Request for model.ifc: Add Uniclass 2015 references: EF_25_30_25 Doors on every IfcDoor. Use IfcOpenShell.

First a look at what the model holds.

```python
import ifcopenshell

model = ifcopenshell.open("model.ifc")
print(model.schema)
print("classifications:", [c.Name for c in model.by_type("IfcClassification")])
for ifc_class in ("IfcDoor", "IfcRoof", "IfcStair", "IfcWall", "IfcWindow"):
    print(ifc_class, len(model.by_type(ifc_class)))
```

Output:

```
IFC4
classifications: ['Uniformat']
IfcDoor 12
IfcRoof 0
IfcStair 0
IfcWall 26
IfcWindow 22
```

```python
import ifcopenshell
import ifcopenshell.api.classification

model = ifcopenshell.open("model.ifc")

system = ifcopenshell.api.classification.add_classification(model, classification="Uniclass 2015")

codes = {
    "IfcDoor": ("EF_25_30_25", "Doors"),
}
for ifc_class, (code, name) in codes.items():
    products = model.by_type(ifc_class)
    ifcopenshell.api.classification.add_reference(
        model, products=products, classification=system, identification=code, name=name
    )
    print(code, len(products))

model.write("model_v2.ifc")
```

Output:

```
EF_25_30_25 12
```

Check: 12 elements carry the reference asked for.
